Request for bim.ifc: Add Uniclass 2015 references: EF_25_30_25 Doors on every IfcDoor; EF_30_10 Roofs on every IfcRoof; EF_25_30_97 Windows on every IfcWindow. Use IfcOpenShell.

First a look at what the model holds.

```python
import ifcopenshell

model = ifcopenshell.open("bim.ifc")
print(model.schema)
print("classifications:", [c.Name for c in model.by_type("IfcClassification")])
for ifc_class in ("IfcDoor", "IfcRoof", "IfcStair", "IfcWall", "IfcWindow"):
    print(ifc_class, len(model.by_type(ifc_class)))
```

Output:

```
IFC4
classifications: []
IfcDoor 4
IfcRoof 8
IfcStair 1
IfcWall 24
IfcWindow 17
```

```python
import ifcopenshell
import ifcopenshell.api.classification

model = ifcopenshell.open("bim.ifc")

system = ifcopenshell.api.classification.add_classification(model, classification="Uniclass 2015")

codes = {
    "IfcDoor": ("EF_25_30_25", "Doors"),
    "IfcRoof": ("EF_30_10", "Roofs"),
    "IfcWindow": ("EF_25_30_97", "Windows"),
}
for ifc_class, (code, name) in codes.items():
    products = model.by_type(ifc_class)
    ifcopenshell.api.classification.add_reference(
        model, products=products, classification=system, identification=code, name=name
    )
    print(code, len(products))

model.write("bim_rev.ifc")
```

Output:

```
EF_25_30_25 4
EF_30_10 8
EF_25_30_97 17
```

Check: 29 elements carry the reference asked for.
